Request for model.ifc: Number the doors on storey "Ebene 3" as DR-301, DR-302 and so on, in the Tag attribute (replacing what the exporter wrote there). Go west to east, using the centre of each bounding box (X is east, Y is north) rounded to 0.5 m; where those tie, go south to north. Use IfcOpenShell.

First a look at what the model holds.

```python
import ifcopenshell
import ifcopenshell.util.element
import ifcopenshell.util.placement

model = ifcopenshell.open("model.ifc")
print(model.schema)
storey = next(s for s in model.by_type("IfcBuildingStorey") if s.Name == "Ebene 3")
doors = [e for e in ifcopenshell.util.element.get_decomposition(storey) if e.is_a("IfcDoor")]
for e in sorted(doors, key=lambda e: e.id()):
    origin = ifcopenshell.util.placement.get_local_placement(e.ObjectPlacement)[:3, 3]
    print(e.id(), e.Tag, e.Name, origin.round(2) + 0.0, sep=" | ")
```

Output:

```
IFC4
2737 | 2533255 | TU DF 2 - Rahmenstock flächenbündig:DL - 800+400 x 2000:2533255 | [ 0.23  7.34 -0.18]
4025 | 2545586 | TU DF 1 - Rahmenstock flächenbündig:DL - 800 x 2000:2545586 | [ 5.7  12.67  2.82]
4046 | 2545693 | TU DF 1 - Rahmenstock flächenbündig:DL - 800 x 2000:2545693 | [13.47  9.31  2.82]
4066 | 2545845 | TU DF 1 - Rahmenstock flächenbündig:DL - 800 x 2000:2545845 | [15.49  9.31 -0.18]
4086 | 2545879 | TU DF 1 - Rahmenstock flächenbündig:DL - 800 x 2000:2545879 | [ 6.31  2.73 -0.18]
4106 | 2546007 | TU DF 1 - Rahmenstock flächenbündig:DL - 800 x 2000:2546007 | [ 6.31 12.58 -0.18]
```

```python
import ifcopenshell
import ifcopenshell.geom
import ifcopenshell.util.element
import ifcopenshell.util.shape

model = ifcopenshell.open("model.ifc")
settings = ifcopenshell.geom.settings()
settings.set("use-world-coords", True)


def centre(element):
    shape = ifcopenshell.geom.create_shape(settings, element)
    return ifcopenshell.util.shape.get_bbox_centroid(shape.geometry)


storey = next(s for s in model.by_type("IfcBuildingStorey") if s.Name == "Ebene 3")
doors = [e for e in ifcopenshell.util.element.get_decomposition(storey) if e.is_a("IfcDoor")]

# Insertion points can sit at a corner or the storey origin, so sort by the geometry (in metres).
centres = {e: centre(e) for e in doors}
doors.sort(key=lambda e: (round(centres[e][0] / 0.5), centres[e][1]))

for i, e in enumerate(doors, start=1):
    number = f"DR-3{i:02d}"
    e.Tag = number
    print(e.id(), number)

model.write("model_v2.ifc")
```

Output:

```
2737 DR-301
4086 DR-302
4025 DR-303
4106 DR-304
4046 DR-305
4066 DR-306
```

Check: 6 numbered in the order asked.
